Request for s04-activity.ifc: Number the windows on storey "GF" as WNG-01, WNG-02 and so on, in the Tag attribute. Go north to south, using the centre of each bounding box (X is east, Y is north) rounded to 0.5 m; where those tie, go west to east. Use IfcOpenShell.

First a look at what the model holds.

```python
import ifcopenshell
import ifcopenshell.util.element
import ifcopenshell.util.placement

model = ifcopenshell.open("s04-activity.ifc")
print(model.schema)
storey = next(s for s in model.by_type("IfcBuildingStorey") if s.Name == "GF")
windows = [e for e in ifcopenshell.util.element.get_decomposition(storey) if e.is_a("IfcWindow")]
for e in sorted(windows, key=lambda e: e.id()):
    origin = ifcopenshell.util.placement.get_local_placement(e.ObjectPlacement)[:3, 3]
    print(e.id(), e.Tag, e.Name, origin.round(2) + 0.0, sep=" | ")
```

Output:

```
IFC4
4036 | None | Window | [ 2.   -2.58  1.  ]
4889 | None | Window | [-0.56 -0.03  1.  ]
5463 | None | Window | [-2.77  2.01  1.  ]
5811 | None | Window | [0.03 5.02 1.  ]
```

```python
import ifcopenshell
import ifcopenshell.geom
import ifcopenshell.util.element
import ifcopenshell.util.shape

model = ifcopenshell.open("s04-activity.ifc")
settings = ifcopenshell.geom.settings()
settings.set("use-world-coords", True)


def centre(element):
    shape = ifcopenshell.geom.create_shape(settings, element)
    return ifcopenshell.util.shape.get_bbox_centroid(shape.geometry)


storey = next(s for s in model.by_type("IfcBuildingStorey") if s.Name == "GF")
windows = [e for e in ifcopenshell.util.element.get_decomposition(storey) if e.is_a("IfcWindow")]

# Insertion points can sit at a corner or the storey origin, so sort by the geometry (in metres).
centres = {e: centre(e) for e in windows}
windows.sort(key=lambda e: (-round(centres[e][1] / 0.5), centres[e][0]))

for i, e in enumerate(windows, start=1):
    number = f"WNG-{i:02d}"
    e.Tag = number
    print(e.id(), number)

model.write("s04-activity_edited.ifc")
```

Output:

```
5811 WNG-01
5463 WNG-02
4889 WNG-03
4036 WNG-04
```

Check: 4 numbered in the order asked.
